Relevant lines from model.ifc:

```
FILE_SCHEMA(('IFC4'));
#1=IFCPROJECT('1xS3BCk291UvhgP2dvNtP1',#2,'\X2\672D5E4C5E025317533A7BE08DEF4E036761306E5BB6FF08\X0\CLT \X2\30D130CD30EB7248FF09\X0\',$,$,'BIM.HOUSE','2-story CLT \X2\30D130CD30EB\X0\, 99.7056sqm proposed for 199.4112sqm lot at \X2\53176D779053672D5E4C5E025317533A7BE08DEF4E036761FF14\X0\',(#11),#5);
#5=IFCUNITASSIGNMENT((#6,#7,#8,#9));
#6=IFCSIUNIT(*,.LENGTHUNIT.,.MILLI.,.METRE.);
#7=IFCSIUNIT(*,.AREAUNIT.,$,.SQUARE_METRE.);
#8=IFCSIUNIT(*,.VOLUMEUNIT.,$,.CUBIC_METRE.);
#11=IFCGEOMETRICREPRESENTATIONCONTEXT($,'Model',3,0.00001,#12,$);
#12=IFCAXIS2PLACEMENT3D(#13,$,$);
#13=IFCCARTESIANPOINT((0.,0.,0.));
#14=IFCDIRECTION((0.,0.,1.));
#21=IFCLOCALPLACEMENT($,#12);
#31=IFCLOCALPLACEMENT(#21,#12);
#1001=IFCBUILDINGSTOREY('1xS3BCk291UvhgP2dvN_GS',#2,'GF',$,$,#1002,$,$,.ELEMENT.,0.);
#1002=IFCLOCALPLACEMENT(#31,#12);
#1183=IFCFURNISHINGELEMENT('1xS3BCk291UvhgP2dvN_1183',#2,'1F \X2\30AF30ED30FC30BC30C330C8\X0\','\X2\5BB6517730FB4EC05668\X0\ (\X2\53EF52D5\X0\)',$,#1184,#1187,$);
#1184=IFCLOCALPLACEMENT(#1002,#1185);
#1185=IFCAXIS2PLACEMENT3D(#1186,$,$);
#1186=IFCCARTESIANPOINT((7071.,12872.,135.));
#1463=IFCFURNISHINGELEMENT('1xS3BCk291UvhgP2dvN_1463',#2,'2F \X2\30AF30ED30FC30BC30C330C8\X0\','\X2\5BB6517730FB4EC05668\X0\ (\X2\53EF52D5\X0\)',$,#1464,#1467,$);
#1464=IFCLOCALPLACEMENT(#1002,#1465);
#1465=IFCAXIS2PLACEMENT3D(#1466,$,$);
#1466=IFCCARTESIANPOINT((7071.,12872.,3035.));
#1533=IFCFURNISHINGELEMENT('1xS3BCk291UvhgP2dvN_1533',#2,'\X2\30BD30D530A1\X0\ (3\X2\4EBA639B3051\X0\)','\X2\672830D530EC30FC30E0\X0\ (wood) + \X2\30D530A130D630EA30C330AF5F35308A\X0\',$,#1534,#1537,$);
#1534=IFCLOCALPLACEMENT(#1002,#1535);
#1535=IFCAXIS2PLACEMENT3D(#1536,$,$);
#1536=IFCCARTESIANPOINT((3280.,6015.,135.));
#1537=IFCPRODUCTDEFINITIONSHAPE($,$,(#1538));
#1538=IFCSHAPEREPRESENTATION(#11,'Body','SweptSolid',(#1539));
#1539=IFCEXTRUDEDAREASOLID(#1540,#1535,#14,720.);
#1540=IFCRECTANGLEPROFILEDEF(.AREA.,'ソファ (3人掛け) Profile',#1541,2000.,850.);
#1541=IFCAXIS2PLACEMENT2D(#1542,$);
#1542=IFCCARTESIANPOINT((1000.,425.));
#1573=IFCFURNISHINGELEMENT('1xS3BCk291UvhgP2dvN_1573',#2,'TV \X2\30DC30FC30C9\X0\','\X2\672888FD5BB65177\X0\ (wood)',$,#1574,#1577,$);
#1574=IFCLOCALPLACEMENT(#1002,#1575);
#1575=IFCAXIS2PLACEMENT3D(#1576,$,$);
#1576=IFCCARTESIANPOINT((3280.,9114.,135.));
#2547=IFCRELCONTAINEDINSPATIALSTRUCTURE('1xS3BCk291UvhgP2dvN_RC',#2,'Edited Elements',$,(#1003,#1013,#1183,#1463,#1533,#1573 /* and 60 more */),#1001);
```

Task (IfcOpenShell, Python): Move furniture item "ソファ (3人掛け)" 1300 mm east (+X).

```python
import ifcopenshell
import ifcopenshell.api.geometry
import ifcopenshell.util.placement
import ifcopenshell.util.unit

model = ifcopenshell.open("model.ifc")
unit_scale = ifcopenshell.util.unit.calculate_unit_scale(model)

item = model.by_id(1533)
matrix = ifcopenshell.util.placement.get_local_placement(item.ObjectPlacement)
matrix[0, 3] += 1.3 / unit_scale
ifcopenshell.api.geometry.edit_object_placement(model, product=item, matrix=matrix, is_si=False)

print(ifcopenshell.util.placement.get_local_placement(item.ObjectPlacement).round(3) + 0.0)

model.write("model-out.ifc")
```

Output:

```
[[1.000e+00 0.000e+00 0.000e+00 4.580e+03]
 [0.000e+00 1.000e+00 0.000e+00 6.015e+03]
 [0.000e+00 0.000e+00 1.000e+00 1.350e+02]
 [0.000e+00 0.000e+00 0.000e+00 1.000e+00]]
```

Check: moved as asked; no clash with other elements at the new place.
